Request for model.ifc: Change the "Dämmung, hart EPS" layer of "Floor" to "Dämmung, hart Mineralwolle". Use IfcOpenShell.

First a look at what the model holds.

```python
import ifcopenshell
import ifcopenshell.util.element

model = ifcopenshell.open("model.ifc")
print(model.schema)
for layer_set in model.by_type("IfcMaterialLayerSet"):
    if layer_set.LayerSetName == "Floor":
        for layer in layer_set.MaterialLayers:
            print(layer.id(), layer.Material and layer.Material.Name, layer.LayerThickness, sep=" | ")
        print(len(ifcopenshell.util.element.get_elements_by_material(model, layer_set)), "elements and types use it")
print(sorted(m.Name for m in model.by_type("IfcMaterial") if m.Name)[:60])
```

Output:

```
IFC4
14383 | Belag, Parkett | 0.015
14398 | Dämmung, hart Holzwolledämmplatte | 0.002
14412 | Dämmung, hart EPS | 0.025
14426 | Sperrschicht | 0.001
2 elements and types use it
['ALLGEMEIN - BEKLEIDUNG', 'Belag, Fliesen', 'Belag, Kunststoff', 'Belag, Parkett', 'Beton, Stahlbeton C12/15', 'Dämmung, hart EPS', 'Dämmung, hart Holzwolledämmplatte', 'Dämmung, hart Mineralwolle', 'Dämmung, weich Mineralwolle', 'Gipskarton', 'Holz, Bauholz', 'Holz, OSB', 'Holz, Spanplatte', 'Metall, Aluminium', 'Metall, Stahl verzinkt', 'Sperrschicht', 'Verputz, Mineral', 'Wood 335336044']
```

```python
import ifcopenshell
import ifcopenshell.api.material

model = ifcopenshell.open("model.ifc")

layer_set = next(s for s in model.by_type("IfcMaterialLayerSet") if s.LayerSetName == "Floor")
layer = next(l for l in layer_set.MaterialLayers if l.Material and l.Material.Name == "Dämmung, hart EPS")
material = next(m for m in model.by_type("IfcMaterial") if m.Name == "Dämmung, hart Mineralwolle")

# Point this one layer at the other material; renaming the old one would change it everywhere.
ifcopenshell.api.material.edit_layer(model, layer=layer, attributes={}, material=material)

print([l.Material.Name if l.Material else None for l in layer_set.MaterialLayers])

model.write("model_edited.ifc")
```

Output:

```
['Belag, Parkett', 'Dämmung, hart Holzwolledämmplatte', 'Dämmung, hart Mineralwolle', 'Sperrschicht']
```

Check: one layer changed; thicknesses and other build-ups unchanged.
